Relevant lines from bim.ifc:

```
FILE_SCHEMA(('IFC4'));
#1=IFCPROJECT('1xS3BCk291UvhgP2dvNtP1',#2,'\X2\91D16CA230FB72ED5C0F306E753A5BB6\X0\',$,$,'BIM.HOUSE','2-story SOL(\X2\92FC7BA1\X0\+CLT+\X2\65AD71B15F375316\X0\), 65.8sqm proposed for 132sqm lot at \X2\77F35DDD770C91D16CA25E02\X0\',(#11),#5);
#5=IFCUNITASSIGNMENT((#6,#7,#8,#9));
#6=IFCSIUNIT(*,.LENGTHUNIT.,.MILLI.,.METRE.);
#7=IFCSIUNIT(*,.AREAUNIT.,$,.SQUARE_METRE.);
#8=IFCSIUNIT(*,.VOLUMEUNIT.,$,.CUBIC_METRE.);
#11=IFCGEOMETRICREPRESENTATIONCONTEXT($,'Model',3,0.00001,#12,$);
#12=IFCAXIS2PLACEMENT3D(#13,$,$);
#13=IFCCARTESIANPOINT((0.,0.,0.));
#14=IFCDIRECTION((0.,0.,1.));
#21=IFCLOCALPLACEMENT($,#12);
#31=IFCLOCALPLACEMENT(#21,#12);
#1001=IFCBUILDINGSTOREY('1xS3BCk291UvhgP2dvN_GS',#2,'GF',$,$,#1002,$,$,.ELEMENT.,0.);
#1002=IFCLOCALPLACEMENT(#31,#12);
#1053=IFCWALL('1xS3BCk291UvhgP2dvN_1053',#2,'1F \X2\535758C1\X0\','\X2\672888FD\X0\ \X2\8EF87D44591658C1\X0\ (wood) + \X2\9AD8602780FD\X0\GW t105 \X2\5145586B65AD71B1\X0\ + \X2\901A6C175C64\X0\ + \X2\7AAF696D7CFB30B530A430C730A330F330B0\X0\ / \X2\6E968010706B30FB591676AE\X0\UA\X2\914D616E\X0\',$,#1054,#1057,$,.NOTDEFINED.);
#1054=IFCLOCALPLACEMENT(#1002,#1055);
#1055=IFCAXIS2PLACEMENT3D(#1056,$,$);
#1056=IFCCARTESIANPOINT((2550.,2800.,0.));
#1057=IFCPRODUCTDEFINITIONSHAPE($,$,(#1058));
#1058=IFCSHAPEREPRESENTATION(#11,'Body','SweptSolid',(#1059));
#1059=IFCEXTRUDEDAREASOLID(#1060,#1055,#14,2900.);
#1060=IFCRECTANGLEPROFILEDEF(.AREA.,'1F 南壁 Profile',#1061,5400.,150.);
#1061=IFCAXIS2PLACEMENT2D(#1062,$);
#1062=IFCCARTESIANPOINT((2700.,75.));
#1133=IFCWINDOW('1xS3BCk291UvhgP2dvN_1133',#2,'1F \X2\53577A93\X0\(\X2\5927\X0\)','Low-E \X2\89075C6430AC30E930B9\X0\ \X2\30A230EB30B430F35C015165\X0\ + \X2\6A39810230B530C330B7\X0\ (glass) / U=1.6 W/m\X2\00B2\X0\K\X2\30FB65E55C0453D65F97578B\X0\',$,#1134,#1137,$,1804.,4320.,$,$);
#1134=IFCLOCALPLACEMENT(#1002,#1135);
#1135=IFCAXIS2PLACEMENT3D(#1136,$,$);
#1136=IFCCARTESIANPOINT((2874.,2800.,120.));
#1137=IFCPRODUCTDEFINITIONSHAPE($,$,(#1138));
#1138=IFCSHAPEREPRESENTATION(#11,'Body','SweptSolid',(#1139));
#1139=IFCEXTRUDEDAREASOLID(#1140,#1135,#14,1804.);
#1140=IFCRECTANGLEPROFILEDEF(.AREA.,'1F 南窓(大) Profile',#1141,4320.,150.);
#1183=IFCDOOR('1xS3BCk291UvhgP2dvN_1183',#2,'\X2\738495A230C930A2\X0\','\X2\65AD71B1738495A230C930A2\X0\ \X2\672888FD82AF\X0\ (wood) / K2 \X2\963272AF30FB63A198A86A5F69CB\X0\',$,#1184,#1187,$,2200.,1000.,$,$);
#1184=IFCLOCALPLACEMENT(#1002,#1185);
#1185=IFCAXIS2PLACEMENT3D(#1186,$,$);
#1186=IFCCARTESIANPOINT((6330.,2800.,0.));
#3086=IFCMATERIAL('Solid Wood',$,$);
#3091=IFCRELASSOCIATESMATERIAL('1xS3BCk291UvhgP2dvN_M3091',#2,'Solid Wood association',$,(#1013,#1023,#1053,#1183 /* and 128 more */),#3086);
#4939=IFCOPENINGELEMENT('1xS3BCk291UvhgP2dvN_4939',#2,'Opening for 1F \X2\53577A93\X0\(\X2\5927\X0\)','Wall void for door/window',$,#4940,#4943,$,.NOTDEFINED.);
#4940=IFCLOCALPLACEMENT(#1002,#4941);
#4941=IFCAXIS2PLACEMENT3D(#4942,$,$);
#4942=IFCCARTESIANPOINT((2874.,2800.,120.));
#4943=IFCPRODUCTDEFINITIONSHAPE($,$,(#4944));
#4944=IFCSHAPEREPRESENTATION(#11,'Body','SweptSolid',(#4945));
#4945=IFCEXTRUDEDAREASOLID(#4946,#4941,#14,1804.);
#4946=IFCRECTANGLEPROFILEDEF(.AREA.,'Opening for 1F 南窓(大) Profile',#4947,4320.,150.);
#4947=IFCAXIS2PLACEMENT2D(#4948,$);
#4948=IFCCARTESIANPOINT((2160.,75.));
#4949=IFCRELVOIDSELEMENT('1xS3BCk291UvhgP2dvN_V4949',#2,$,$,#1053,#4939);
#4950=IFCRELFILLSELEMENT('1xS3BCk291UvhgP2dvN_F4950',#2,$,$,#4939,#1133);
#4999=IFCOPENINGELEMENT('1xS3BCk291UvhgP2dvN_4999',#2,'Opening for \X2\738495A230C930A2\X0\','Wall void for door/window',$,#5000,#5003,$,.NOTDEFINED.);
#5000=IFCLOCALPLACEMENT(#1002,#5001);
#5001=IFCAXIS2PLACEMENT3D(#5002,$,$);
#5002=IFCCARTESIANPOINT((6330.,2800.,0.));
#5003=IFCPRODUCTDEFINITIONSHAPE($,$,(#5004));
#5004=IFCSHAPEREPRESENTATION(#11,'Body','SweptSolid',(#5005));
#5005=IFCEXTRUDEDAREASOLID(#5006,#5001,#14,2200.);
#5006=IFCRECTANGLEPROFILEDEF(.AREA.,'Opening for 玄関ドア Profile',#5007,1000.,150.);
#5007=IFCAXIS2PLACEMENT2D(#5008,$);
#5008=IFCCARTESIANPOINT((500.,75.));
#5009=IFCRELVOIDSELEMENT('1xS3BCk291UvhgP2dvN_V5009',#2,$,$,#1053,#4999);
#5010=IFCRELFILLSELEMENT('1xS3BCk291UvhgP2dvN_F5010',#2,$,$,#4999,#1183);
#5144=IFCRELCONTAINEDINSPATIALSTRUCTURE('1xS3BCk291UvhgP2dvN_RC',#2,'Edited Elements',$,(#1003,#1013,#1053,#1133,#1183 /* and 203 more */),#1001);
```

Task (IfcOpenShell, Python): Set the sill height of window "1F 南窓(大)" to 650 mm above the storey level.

```python
import numpy as np
import ifcopenshell
import ifcopenshell.api.geometry
import ifcopenshell.geom
import ifcopenshell.util.element
import ifcopenshell.util.placement
import ifcopenshell.util.shape
import ifcopenshell.util.unit

model = ifcopenshell.open("bim.ifc")
unit_scale = ifcopenshell.util.unit.calculate_unit_scale(model)

window = model.by_id(1133)
opening = window.FillsVoids[0].RelatingOpeningElement
storey = ifcopenshell.util.element.get_container(window, ifc_class="IfcBuildingStorey")
level = ifcopenshell.util.placement.get_local_placement(storey.ObjectPlacement)[2, 3]

# The opening's origin need not be at the sill, so measure its lowest point.
shape = ifcopenshell.geom.create_shape(ifcopenshell.geom.settings(), opening)
bottom = ifcopenshell.util.shape.get_shape_bottom_elevation(shape, shape.geometry) / unit_scale
dz = level + 650.0 - bottom

shift = np.array([0.0, 0.0, dz])
# The window is not placed relative to its opening, so move both.
for product in (opening, window):
    matrix = ifcopenshell.util.placement.get_local_placement(product.ObjectPlacement)
    matrix[:3, 3] += shift
    ifcopenshell.api.geometry.edit_object_placement(model, product=product, matrix=matrix, is_si=False)

print(f"moved by {dz * unit_scale:+.3f} m")

model.write("bim_rev.ifc")
```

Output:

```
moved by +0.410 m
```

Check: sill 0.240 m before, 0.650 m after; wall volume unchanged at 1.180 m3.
